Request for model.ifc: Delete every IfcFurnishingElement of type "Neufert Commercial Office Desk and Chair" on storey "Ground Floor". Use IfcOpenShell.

First a look at what the model holds.

```python
import ifcopenshell
import ifcopenshell.util.element

model = ifcopenshell.open("model.ifc")
print(model.schema)
storey = next(s for s in model.by_type("IfcBuildingStorey") if s.Name == "Ground Floor")
furniture = [e for e in ifcopenshell.util.element.get_decomposition(storey) if e.is_a("IfcFurnishingElement")]
seen = {}
for e in furniture:
    element_type = ifcopenshell.util.element.get_type(e)
    name = element_type.Name if element_type not in (None, e) else None
    seen[name] = seen.get(name, 0) + 1
for name, count in sorted(seen.items(), key=str):
    print(count, "x", name)
```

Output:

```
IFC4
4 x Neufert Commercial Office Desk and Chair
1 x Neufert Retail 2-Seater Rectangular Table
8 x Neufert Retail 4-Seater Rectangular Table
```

```python
import ifcopenshell
import ifcopenshell.api.root
import ifcopenshell.util.element

model = ifcopenshell.open("model.ifc")

storey = next(s for s in model.by_type("IfcBuildingStorey") if s.Name == "Ground Floor")
furniture = [e for e in ifcopenshell.util.element.get_decomposition(storey) if e.is_a("IfcFurnishingElement")]
targets = [e for e in furniture if (t := ifcopenshell.util.element.get_type(e)) not in (None, e) and t.Name == "Neufert Commercial Office Desk and Chair"]

for e in targets:
    ifcopenshell.api.root.remove_product(model, product=e)
print(len(targets), "removed")

model.write("model-out.ifc")
```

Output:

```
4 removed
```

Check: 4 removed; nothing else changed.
